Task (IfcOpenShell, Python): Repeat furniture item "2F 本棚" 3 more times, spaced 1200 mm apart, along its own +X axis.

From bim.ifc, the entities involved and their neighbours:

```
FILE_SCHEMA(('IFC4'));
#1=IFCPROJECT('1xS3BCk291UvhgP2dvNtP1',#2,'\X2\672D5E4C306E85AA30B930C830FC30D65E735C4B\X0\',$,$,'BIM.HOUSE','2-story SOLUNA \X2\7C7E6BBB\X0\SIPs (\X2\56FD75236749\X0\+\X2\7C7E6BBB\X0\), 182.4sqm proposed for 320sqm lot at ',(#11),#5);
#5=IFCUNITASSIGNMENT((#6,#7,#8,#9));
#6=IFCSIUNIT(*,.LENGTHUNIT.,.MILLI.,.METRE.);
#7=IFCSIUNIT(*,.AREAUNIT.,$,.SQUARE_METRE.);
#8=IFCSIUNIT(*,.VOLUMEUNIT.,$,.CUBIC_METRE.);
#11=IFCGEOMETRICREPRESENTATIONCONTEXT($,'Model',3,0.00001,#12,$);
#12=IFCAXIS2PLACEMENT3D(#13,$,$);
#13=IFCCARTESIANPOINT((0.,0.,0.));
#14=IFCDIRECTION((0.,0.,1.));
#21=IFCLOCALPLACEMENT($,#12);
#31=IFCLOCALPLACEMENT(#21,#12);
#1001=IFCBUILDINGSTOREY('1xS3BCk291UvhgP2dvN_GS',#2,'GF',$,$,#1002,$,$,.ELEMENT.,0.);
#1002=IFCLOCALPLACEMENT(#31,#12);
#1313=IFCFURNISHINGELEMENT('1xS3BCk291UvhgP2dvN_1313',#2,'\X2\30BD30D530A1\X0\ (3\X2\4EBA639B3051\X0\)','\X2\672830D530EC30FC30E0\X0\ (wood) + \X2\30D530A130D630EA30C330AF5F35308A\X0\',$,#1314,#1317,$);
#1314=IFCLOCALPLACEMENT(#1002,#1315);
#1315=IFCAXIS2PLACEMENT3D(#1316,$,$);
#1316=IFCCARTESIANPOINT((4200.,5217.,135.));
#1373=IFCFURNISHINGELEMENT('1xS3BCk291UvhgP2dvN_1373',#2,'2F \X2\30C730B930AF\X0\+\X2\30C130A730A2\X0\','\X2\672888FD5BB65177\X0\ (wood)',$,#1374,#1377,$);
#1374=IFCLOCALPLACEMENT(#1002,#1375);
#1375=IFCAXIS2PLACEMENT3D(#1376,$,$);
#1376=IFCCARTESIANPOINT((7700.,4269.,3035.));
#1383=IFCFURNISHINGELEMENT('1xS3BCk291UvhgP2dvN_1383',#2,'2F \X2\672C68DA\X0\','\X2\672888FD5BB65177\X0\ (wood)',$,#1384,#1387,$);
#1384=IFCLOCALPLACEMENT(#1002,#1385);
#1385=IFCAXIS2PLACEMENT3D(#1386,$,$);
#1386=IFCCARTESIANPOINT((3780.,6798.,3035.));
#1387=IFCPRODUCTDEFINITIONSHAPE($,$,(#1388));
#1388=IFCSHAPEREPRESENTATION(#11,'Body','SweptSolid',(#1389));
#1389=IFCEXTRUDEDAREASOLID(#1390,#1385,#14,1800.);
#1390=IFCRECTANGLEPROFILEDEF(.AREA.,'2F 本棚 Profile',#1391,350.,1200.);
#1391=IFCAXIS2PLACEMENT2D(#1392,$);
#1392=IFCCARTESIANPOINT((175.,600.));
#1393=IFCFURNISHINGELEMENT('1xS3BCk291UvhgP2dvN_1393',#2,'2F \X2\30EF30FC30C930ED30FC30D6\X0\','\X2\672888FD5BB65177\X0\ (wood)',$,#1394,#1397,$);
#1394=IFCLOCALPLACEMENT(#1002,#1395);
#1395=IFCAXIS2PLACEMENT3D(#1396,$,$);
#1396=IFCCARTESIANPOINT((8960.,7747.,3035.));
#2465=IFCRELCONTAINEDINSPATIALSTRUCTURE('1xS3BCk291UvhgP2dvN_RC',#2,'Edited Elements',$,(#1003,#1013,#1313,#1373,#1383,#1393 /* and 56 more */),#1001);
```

```python
import ifcopenshell
import ifcopenshell.api.geometry
import ifcopenshell.api.root
import ifcopenshell.util.element
import ifcopenshell.util.placement
import ifcopenshell.util.unit

model = ifcopenshell.open("bim.ifc")
unit_scale = ifcopenshell.util.unit.calculate_unit_scale(model)


def reuse_history(source, copy):
    """copy_class also copies each property set's owner history, people and application; keep the originals."""
    for rel in copy.IsDefinedBy:
        if rel.is_a("IfcRelDefinesByProperties") and (history := rel.RelatingPropertyDefinition.OwnerHistory):
            rel.RelatingPropertyDefinition.OwnerHistory = source.OwnerHistory
            ifcopenshell.util.element.remove_deep2(model, history)


source = model.by_id(1383)
base = ifcopenshell.util.placement.get_local_placement(source.ObjectPlacement)
step = base[:3, 0] * 1.2 / unit_scale

for i in range(1, 4):
    copy = ifcopenshell.api.root.copy_class(model, product=source)
    copy.Representation = ifcopenshell.util.element.copy_deep(
        model, source.Representation, exclude=["IfcGeometricRepresentationContext", "IfcRepresentationMap"]
    )
    reuse_history(source, copy)
    matrix = base.copy()
    matrix[:3, 3] += i * step
    print("added at", matrix[:3, 3].round(3) + 0.0)
    ifcopenshell.api.geometry.edit_object_placement(model, product=copy, matrix=matrix, is_si=False)

model.write("bim_v2.ifc")
```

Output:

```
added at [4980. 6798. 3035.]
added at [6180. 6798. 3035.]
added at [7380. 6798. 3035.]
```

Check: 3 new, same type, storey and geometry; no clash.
